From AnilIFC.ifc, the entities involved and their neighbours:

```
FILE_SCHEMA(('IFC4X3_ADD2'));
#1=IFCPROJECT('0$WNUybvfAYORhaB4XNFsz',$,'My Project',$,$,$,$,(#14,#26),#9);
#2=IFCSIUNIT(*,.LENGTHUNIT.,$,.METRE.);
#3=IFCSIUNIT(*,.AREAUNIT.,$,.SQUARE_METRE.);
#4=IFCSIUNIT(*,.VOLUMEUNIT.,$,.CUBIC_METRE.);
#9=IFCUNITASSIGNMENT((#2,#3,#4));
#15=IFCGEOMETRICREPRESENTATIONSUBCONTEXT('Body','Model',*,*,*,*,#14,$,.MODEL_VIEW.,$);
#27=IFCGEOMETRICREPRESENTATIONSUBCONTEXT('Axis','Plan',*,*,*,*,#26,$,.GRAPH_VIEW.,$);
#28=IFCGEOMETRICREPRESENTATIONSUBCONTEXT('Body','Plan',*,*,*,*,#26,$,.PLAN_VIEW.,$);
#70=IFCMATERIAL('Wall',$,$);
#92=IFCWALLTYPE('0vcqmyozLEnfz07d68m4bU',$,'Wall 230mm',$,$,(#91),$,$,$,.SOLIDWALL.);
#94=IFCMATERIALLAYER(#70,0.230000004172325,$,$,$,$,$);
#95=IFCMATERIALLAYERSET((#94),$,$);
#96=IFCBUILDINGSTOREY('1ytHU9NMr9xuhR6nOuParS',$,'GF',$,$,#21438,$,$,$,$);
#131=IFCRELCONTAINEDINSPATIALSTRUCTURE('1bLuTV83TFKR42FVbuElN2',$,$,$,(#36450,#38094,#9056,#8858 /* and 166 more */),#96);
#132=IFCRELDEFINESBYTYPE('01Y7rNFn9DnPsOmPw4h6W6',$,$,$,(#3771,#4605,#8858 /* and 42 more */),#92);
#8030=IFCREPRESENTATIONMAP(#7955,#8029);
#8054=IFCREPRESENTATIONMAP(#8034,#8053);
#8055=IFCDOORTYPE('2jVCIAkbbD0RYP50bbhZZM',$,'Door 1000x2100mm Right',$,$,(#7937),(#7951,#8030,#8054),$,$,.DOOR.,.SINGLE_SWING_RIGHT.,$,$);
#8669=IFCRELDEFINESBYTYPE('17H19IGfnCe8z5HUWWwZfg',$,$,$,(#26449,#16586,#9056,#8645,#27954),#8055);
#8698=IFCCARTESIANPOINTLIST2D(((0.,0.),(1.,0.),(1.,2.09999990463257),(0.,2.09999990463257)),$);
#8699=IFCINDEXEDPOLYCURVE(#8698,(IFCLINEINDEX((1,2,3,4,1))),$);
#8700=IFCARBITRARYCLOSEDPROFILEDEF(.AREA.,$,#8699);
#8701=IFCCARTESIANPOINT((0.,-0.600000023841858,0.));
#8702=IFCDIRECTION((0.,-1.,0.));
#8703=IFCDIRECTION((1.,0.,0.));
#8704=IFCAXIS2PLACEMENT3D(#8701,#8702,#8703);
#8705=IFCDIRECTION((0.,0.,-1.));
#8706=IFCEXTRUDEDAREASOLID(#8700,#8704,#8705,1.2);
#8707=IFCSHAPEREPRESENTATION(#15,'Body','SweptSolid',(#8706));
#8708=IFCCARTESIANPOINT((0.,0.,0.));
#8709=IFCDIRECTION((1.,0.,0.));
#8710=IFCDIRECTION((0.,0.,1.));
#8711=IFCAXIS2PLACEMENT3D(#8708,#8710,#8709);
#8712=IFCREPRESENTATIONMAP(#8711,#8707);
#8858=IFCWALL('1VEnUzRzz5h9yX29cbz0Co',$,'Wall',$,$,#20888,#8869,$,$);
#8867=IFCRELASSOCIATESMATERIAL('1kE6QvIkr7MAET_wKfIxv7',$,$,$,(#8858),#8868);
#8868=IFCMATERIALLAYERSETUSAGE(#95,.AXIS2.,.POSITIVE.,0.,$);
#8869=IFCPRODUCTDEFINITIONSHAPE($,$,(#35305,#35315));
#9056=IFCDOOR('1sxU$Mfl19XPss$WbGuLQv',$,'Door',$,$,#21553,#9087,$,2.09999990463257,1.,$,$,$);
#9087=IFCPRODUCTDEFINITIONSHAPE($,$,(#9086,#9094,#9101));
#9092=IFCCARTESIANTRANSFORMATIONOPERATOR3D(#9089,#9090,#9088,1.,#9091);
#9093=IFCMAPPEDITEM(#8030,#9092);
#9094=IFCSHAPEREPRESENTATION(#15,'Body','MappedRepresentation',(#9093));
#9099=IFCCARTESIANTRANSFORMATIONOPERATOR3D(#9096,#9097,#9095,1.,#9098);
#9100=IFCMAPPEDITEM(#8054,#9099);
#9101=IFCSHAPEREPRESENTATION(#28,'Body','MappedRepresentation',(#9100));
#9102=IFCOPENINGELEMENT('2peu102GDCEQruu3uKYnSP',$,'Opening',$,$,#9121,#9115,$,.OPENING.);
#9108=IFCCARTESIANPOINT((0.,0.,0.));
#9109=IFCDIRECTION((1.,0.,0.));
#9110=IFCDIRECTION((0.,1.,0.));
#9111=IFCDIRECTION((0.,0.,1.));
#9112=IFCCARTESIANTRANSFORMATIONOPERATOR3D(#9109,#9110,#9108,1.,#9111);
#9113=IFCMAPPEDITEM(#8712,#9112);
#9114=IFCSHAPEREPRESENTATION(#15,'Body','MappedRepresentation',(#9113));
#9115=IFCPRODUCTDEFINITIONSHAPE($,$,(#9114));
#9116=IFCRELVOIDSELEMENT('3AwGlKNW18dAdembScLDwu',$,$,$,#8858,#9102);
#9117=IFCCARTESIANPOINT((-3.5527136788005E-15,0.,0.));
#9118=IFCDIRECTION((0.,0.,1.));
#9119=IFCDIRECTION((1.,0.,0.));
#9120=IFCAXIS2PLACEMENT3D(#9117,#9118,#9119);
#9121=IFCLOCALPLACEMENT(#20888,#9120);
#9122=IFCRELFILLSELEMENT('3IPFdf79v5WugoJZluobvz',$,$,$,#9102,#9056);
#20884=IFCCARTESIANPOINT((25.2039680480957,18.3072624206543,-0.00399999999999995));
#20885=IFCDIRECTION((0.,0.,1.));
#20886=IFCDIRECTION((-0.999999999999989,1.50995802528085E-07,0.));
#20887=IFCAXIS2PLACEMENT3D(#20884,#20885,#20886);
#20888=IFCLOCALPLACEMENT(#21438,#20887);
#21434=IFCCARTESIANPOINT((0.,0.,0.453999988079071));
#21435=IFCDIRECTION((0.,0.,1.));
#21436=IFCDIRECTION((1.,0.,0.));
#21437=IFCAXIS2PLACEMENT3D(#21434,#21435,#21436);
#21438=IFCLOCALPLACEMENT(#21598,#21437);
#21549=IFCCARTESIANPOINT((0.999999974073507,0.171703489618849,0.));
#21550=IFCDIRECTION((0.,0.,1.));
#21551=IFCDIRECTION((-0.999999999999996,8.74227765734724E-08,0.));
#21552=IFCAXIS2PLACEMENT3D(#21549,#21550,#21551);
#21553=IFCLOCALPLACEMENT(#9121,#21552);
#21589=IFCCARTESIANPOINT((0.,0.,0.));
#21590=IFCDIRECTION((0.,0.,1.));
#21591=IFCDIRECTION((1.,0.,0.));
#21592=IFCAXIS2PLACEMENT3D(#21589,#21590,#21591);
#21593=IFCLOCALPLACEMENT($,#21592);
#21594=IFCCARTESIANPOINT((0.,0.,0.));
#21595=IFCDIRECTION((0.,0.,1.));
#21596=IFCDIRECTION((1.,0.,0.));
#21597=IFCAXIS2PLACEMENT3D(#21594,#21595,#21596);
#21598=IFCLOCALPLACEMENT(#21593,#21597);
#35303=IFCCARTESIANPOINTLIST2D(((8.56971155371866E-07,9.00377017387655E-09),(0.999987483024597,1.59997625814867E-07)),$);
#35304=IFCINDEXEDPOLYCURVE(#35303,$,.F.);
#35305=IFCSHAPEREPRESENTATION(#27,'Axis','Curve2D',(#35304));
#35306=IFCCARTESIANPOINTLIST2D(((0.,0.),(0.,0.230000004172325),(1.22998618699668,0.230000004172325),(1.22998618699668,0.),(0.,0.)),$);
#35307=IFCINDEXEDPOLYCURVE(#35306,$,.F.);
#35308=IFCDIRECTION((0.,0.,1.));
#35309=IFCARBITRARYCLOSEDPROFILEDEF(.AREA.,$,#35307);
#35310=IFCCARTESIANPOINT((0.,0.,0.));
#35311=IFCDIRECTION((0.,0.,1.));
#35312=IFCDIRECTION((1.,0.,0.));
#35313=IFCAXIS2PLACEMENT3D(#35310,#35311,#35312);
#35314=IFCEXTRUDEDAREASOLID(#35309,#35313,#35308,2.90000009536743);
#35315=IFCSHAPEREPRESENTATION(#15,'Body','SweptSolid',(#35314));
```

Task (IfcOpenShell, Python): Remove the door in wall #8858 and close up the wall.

```python
import ifcopenshell
import ifcopenshell.api.feature
import ifcopenshell.api.root
import ifcopenshell.geom
import ifcopenshell.util.shape

model = ifcopenshell.open("AnilIFC.ifc")
settings = ifcopenshell.geom.settings()


def volume(element):
    """Net volume in cubic metres, openings subtracted."""
    shape = ifcopenshell.geom.create_shape(settings, element)
    return ifcopenshell.util.shape.get_volume(shape.geometry)


door = model.by_guid("1sxU$Mfl19XPss$WbGuLQv")
opening = door.FillsVoids[0].RelatingOpeningElement
wall = opening.VoidsElements[0].RelatingBuildingElement
before = volume(wall)

ifcopenshell.api.root.remove_product(model, product=door)
ifcopenshell.api.feature.remove_feature(model, feature=opening)

after = volume(wall)

print(f"wall volume {before:.3f} -> {after:.3f} m3")

model.write("AnilIFC_updated.ifc")
```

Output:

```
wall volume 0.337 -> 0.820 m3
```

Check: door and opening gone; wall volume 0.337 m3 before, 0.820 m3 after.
